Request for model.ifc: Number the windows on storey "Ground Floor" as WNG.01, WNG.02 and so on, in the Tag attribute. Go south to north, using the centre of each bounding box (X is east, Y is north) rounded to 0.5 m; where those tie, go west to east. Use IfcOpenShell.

First a look at what the model holds.

```python
import ifcopenshell
import ifcopenshell.util.element
import ifcopenshell.util.placement

model = ifcopenshell.open("model.ifc")
print(model.schema)
storey = next(s for s in model.by_type("IfcBuildingStorey") if s.Name == "Ground Floor")
windows = [e for e in ifcopenshell.util.element.get_decomposition(storey) if e.is_a("IfcWindow")]
for e in sorted(windows, key=lambda e: e.id()):
    origin = ifcopenshell.util.placement.get_local_placement(e.ObjectPlacement)[:3, 3]
    print(e.id(), e.Tag, e.Name, origin.round(2) + 0.0, sep=" | ")
```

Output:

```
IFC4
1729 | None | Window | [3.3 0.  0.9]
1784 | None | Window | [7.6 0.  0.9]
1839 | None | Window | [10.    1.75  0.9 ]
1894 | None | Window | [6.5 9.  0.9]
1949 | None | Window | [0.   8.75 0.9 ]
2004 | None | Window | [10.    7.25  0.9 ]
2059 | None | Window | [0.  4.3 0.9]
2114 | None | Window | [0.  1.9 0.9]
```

```python
import ifcopenshell
import ifcopenshell.geom
import ifcopenshell.util.element
import ifcopenshell.util.shape

model = ifcopenshell.open("model.ifc")
settings = ifcopenshell.geom.settings()
settings.set("use-world-coords", True)


def centre(element):
    shape = ifcopenshell.geom.create_shape(settings, element)
    return ifcopenshell.util.shape.get_bbox_centroid(shape.geometry)


storey = next(s for s in model.by_type("IfcBuildingStorey") if s.Name == "Ground Floor")
windows = [e for e in ifcopenshell.util.element.get_decomposition(storey) if e.is_a("IfcWindow")]

# Insertion points can sit at a corner or the storey origin, so sort by the geometry (in metres).
centres = {e: centre(e) for e in windows}
windows.sort(key=lambda e: (round(centres[e][1] / 0.5), centres[e][0]))

for i, e in enumerate(windows, start=1):
    number = f"WNG.{i:02d}"
    e.Tag = number
    print(e.id(), number)

model.write("model_rev.ifc")
```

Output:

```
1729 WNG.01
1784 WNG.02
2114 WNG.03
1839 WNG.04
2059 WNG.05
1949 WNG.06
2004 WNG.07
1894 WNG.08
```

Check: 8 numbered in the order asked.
